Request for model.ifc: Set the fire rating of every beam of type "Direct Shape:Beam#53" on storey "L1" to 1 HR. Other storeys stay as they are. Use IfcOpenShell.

First a look at what the model holds.

```python
import ifcopenshell
import ifcopenshell.util.element

model = ifcopenshell.open("model.ifc")
print(model.schema)
storey = next(s for s in model.by_type("IfcBuildingStorey") if s.Name == "L1")
beams = [e for e in ifcopenshell.util.element.get_decomposition(storey) if e.is_a("IfcBeam")]
seen = {}
for e in beams:
    element_type = ifcopenshell.util.element.get_type(e)
    key = (element_type.Name if element_type != e and element_type else None, ifcopenshell.util.element.get_pset(e, "Pset_BeamCommon", "FireRating"))
    seen[key] = seen.get(key, 0) + 1
for (name, value), count in sorted(seen.items(), key=str):
    print(count, "x", name, "|", value)
```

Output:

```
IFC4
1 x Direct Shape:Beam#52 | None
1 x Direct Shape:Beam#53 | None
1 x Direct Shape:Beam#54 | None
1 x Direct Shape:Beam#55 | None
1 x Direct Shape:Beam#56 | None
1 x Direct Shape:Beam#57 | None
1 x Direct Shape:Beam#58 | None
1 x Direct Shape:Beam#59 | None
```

```python
import ifcopenshell
import ifcopenshell.api.pset
import ifcopenshell.util.element

model = ifcopenshell.open("model.ifc")

storey = next(s for s in model.by_type("IfcBuildingStorey") if s.Name == "L1")
beams = [e for e in ifcopenshell.util.element.get_decomposition(storey) if e.is_a("IfcBeam")]

count = 0
for e in beams:
    element_type = ifcopenshell.util.element.get_type(e)
    if element_type in (None, e) or element_type.Name != "Direct Shape:Beam#53":
        continue
    # add_pset returns the element's existing set when there is one.
    pset = ifcopenshell.api.pset.add_pset(model, product=e, name="Pset_BeamCommon")
    ifcopenshell.api.pset.edit_pset(model, pset=pset, properties={"FireRating": "1 HR"})
    count += 1

print(count, "beams updated")

model.write("model_edited.ifc")
```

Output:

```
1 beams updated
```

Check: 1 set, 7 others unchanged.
